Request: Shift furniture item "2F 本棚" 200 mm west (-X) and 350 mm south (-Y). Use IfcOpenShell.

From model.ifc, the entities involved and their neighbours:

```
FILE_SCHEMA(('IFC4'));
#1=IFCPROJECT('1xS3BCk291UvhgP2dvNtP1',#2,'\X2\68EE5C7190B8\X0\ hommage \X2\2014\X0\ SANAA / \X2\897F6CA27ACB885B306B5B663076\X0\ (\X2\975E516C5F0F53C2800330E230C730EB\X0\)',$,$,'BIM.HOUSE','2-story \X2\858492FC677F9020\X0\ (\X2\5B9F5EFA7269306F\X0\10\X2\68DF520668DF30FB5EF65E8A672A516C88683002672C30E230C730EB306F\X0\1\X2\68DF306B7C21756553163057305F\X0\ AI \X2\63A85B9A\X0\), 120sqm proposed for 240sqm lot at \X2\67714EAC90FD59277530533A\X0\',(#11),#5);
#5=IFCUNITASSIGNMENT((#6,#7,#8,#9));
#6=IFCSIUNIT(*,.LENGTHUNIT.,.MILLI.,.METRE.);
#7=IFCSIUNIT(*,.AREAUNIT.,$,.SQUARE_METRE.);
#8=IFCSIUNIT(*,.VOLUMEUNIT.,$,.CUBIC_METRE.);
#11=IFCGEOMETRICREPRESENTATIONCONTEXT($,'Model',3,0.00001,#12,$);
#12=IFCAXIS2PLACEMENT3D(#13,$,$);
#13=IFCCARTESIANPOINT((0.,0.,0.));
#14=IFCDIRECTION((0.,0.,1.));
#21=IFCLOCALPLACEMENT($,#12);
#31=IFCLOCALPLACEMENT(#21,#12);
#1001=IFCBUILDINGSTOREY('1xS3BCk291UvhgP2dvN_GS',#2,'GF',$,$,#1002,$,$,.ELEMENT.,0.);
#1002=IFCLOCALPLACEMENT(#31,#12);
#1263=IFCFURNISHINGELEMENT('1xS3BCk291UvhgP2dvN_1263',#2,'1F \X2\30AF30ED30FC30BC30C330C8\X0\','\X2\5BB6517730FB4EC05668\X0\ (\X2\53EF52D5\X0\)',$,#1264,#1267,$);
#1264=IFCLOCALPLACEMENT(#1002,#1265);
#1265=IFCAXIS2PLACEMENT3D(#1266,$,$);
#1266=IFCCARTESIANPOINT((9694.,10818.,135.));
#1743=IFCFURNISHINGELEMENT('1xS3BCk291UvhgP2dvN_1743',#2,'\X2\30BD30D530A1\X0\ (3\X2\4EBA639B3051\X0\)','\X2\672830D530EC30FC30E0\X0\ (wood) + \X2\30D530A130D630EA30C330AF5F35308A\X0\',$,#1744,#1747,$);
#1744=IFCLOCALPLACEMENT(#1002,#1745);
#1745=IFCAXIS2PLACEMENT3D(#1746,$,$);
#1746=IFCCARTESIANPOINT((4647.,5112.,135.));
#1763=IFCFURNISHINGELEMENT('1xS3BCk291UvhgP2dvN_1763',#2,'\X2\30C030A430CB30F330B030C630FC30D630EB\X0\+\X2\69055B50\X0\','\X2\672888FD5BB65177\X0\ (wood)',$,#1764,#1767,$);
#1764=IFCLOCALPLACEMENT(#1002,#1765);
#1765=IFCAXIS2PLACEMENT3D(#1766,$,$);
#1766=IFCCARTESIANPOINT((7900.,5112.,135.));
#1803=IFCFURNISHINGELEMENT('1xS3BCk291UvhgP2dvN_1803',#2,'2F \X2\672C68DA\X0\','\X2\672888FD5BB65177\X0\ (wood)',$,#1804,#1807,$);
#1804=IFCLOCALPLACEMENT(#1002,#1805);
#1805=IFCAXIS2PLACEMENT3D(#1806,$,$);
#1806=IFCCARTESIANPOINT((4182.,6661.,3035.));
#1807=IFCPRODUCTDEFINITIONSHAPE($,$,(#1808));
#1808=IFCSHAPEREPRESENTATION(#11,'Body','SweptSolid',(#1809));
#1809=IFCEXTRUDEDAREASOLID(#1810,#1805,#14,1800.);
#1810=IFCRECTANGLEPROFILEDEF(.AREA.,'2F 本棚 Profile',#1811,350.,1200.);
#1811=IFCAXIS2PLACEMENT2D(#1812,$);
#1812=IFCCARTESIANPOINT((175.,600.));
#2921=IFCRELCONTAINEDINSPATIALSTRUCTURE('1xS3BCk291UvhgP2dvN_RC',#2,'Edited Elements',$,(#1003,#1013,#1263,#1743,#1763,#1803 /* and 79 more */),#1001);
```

```python
import ifcopenshell
import ifcopenshell.api.geometry
import ifcopenshell.util.placement
import ifcopenshell.util.unit

model = ifcopenshell.open("model.ifc")
unit_scale = ifcopenshell.util.unit.calculate_unit_scale(model)

item = model.by_guid("1xS3BCk291UvhgP2dvN_1803")
matrix = ifcopenshell.util.placement.get_local_placement(item.ObjectPlacement)
matrix[0, 3] -= 0.2 / unit_scale
matrix[1, 3] -= 0.35 / unit_scale
ifcopenshell.api.geometry.edit_object_placement(model, product=item, matrix=matrix, is_si=False)

print(ifcopenshell.util.placement.get_local_placement(item.ObjectPlacement).round(3) + 0.0)

model.write("model_v2.ifc")
```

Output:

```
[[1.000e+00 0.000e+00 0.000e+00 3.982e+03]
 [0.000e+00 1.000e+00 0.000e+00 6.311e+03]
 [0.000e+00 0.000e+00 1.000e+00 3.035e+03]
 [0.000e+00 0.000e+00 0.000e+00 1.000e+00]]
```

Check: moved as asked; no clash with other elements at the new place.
